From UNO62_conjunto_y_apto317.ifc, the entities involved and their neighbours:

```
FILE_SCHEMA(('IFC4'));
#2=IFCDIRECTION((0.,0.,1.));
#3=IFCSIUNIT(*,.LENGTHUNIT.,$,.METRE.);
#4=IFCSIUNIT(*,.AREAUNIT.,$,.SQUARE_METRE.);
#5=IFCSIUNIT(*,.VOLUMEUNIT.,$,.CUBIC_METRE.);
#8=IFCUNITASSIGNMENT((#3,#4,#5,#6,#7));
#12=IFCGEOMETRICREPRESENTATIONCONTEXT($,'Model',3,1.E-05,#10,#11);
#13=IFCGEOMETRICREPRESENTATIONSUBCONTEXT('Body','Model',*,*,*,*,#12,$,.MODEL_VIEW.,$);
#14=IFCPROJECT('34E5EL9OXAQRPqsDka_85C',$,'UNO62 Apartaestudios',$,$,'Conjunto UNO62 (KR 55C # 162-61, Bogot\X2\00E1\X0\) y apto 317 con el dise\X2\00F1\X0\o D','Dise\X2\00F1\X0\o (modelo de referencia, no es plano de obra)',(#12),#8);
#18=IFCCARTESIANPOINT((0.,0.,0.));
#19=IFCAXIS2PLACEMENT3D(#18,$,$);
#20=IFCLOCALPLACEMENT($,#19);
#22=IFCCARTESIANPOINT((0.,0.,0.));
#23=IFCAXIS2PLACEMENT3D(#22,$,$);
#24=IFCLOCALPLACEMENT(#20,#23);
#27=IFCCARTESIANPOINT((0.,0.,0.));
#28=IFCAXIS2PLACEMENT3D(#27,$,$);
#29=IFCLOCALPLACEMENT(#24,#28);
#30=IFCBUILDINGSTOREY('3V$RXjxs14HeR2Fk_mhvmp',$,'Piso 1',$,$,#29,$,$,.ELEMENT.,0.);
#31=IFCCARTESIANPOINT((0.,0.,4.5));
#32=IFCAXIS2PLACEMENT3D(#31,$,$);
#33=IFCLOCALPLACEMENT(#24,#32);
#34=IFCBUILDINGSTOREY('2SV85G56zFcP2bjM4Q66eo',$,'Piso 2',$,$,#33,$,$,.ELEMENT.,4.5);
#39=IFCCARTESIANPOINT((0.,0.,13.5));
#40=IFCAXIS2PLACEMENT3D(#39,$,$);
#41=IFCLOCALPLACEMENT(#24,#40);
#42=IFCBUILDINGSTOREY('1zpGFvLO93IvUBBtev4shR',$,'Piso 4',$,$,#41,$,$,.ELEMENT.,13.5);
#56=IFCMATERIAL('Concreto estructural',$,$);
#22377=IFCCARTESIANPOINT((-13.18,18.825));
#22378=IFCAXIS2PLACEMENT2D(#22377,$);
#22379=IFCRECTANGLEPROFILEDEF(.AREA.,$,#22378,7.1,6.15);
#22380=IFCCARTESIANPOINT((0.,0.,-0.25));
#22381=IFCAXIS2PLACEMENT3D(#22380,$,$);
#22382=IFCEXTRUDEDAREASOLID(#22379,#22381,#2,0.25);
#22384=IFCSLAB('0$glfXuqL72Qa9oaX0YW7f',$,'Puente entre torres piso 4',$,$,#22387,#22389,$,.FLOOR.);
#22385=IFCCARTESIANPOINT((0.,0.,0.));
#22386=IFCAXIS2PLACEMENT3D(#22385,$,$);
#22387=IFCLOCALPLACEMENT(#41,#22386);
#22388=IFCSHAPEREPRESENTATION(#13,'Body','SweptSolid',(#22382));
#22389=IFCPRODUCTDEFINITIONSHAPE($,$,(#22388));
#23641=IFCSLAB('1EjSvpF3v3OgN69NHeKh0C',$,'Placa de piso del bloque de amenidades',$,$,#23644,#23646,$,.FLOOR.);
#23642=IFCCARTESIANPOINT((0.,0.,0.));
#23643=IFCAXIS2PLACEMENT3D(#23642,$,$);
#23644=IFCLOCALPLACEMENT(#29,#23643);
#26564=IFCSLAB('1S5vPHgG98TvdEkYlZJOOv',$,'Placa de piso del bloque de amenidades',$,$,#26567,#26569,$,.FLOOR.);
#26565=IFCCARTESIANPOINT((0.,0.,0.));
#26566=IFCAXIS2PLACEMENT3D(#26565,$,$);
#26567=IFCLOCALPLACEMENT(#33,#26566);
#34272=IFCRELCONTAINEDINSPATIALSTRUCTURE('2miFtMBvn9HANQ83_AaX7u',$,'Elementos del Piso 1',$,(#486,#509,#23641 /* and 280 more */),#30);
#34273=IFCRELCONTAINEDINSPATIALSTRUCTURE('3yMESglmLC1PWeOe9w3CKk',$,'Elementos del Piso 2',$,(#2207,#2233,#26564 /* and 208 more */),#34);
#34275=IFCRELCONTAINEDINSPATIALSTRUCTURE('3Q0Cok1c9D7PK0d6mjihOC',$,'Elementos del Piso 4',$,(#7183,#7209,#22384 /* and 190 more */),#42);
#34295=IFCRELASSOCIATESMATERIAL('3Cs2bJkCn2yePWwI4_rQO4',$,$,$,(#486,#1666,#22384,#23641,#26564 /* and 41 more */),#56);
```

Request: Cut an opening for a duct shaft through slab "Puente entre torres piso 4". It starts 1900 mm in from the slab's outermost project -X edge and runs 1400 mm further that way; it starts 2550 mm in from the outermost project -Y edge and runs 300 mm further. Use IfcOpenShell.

```python
import numpy as np
import ifcopenshell
import ifcopenshell.api.feature
import ifcopenshell.api.geometry
import ifcopenshell.api.root
import ifcopenshell.geom
import ifcopenshell.util.placement
import ifcopenshell.util.representation
import ifcopenshell.util.shape
import ifcopenshell.util.unit

model = ifcopenshell.open("UNO62_conjunto_y_apto317.ifc")
unit_scale = ifcopenshell.util.unit.calculate_unit_scale(model)
settings = ifcopenshell.geom.settings()


def volume(element):
    """Net volume in cubic metres, openings subtracted."""
    shape = ifcopenshell.geom.create_shape(settings, element)
    return ifcopenshell.util.shape.get_volume(shape.geometry)


slab = model.by_guid("0$glfXuqL72Qa9oaX0YW7f")
before = volume(slab)

# Extent in the slab's own axes, in metres. The edges named are its -X and -Y sides.
slab_shape = ifcopenshell.geom.create_shape(settings, slab)
vertices = ifcopenshell.util.shape.get_vertices(slab_shape.geometry)
x_min, y_min, bottom = vertices.min(axis=0)
top = vertices[:, 2].max()

opening = ifcopenshell.api.root.create_entity(model, ifc_class="IfcOpeningElement", name="Duct shaft opening", predefined_type="OPENING")
context = ifcopenshell.util.representation.get_context(model, "Model", "Body", "MODEL_VIEW")
width, depth = 1.4, 0.3
outline = [(0.0, 0.0), (width, 0.0), (width, depth), (0.0, depth), (0.0, 0.0)]
# Overshoot both faces by 50 mm so the cut is clean.
shape = ifcopenshell.api.geometry.add_slab_representation(
    model, context=context, depth=top - bottom + 0.1, polyline=outline
)
ifcopenshell.api.geometry.assign_representation(model, product=opening, representation=shape)

matrix = ifcopenshell.util.placement.get_local_placement(slab.ObjectPlacement)
matrix[:, 3] = matrix @ np.append(np.array([x_min + 1.9, y_min + 2.55, bottom - 0.05]) / unit_scale, 1.0)
ifcopenshell.api.geometry.edit_object_placement(model, product=opening, matrix=matrix, is_si=False)
ifcopenshell.api.feature.add_feature(model, feature=opening, element=slab)

after = volume(slab)

print(f"slab volume {before:.3f} -> {after:.3f} m3")

model.write("UNO62_conjunto_y_apto317_updated.ifc")
```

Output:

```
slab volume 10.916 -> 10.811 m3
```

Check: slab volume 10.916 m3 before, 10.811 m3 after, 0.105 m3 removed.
